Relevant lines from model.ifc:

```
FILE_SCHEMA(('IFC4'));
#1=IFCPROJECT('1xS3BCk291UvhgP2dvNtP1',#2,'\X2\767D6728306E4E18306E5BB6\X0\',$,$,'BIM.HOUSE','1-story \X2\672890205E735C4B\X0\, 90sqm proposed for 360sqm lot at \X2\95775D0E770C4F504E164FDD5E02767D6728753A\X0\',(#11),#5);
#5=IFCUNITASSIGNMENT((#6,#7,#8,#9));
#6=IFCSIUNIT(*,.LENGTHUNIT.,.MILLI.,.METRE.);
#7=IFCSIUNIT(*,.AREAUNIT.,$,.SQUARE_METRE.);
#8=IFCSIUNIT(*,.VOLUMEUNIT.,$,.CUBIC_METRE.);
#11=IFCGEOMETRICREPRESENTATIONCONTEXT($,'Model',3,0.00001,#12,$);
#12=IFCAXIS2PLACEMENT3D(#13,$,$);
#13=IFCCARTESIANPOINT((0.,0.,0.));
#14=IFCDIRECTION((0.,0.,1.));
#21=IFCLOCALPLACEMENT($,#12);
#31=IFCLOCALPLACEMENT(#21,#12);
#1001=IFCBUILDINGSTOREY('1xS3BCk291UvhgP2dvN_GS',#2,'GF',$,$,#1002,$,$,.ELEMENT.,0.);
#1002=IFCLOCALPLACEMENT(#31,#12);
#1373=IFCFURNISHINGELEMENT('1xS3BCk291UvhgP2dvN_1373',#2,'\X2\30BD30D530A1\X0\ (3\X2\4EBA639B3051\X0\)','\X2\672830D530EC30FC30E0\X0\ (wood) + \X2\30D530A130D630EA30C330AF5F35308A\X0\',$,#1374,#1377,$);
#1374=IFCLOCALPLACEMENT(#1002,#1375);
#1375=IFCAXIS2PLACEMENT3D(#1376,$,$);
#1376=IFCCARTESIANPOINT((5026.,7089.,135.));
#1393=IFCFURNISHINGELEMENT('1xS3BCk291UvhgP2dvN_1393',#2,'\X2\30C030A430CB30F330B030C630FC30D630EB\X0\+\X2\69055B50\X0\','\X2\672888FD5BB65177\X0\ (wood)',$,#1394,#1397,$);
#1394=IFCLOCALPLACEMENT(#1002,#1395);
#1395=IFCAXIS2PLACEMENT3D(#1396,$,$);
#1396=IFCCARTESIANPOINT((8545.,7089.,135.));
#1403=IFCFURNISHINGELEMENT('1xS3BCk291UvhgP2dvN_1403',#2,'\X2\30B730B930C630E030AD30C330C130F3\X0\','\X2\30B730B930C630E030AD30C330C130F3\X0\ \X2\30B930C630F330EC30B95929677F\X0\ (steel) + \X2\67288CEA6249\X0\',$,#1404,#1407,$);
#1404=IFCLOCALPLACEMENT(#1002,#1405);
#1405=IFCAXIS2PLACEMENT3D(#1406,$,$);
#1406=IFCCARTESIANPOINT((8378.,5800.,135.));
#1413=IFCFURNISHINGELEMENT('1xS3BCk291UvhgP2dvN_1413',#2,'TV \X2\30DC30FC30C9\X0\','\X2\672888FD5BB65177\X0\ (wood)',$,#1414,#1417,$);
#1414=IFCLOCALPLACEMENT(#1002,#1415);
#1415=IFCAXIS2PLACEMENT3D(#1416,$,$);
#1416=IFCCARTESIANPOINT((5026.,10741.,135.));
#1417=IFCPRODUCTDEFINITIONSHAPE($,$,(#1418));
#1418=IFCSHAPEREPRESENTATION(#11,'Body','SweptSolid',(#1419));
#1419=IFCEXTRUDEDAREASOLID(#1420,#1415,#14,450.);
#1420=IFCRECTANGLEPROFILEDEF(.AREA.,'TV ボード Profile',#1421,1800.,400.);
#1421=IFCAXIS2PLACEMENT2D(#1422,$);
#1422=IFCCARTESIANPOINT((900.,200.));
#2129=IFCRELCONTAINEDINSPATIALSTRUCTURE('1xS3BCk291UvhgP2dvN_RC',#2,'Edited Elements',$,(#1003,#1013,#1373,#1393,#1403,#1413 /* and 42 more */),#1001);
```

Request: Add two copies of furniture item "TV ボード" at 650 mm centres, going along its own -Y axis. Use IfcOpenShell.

```python
import ifcopenshell
import ifcopenshell.api.geometry
import ifcopenshell.api.root
import ifcopenshell.util.element
import ifcopenshell.util.placement
import ifcopenshell.util.unit

model = ifcopenshell.open("model.ifc")
unit_scale = ifcopenshell.util.unit.calculate_unit_scale(model)


def reuse_history(source, copy):
    """copy_class also copies each property set's owner history, people and application; keep the originals."""
    for rel in copy.IsDefinedBy:
        if rel.is_a("IfcRelDefinesByProperties") and (history := rel.RelatingPropertyDefinition.OwnerHistory):
            rel.RelatingPropertyDefinition.OwnerHistory = source.OwnerHistory
            ifcopenshell.util.element.remove_deep2(model, history)


source = model.by_guid("1xS3BCk291UvhgP2dvN_1413")
base = ifcopenshell.util.placement.get_local_placement(source.ObjectPlacement)
step = -base[:3, 1] * 0.65 / unit_scale

for i in range(1, 3):
    copy = ifcopenshell.api.root.copy_class(model, product=source)
    copy.Representation = ifcopenshell.util.element.copy_deep(
        model, source.Representation, exclude=["IfcGeometricRepresentationContext", "IfcRepresentationMap"]
    )
    reuse_history(source, copy)
    matrix = base.copy()
    matrix[:3, 3] += i * step
    print("added at", matrix[:3, 3].round(3) + 0.0)
    ifcopenshell.api.geometry.edit_object_placement(model, product=copy, matrix=matrix, is_si=False)

model.write("model-out.ifc")
```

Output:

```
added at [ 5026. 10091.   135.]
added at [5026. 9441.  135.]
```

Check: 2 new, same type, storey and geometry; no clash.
